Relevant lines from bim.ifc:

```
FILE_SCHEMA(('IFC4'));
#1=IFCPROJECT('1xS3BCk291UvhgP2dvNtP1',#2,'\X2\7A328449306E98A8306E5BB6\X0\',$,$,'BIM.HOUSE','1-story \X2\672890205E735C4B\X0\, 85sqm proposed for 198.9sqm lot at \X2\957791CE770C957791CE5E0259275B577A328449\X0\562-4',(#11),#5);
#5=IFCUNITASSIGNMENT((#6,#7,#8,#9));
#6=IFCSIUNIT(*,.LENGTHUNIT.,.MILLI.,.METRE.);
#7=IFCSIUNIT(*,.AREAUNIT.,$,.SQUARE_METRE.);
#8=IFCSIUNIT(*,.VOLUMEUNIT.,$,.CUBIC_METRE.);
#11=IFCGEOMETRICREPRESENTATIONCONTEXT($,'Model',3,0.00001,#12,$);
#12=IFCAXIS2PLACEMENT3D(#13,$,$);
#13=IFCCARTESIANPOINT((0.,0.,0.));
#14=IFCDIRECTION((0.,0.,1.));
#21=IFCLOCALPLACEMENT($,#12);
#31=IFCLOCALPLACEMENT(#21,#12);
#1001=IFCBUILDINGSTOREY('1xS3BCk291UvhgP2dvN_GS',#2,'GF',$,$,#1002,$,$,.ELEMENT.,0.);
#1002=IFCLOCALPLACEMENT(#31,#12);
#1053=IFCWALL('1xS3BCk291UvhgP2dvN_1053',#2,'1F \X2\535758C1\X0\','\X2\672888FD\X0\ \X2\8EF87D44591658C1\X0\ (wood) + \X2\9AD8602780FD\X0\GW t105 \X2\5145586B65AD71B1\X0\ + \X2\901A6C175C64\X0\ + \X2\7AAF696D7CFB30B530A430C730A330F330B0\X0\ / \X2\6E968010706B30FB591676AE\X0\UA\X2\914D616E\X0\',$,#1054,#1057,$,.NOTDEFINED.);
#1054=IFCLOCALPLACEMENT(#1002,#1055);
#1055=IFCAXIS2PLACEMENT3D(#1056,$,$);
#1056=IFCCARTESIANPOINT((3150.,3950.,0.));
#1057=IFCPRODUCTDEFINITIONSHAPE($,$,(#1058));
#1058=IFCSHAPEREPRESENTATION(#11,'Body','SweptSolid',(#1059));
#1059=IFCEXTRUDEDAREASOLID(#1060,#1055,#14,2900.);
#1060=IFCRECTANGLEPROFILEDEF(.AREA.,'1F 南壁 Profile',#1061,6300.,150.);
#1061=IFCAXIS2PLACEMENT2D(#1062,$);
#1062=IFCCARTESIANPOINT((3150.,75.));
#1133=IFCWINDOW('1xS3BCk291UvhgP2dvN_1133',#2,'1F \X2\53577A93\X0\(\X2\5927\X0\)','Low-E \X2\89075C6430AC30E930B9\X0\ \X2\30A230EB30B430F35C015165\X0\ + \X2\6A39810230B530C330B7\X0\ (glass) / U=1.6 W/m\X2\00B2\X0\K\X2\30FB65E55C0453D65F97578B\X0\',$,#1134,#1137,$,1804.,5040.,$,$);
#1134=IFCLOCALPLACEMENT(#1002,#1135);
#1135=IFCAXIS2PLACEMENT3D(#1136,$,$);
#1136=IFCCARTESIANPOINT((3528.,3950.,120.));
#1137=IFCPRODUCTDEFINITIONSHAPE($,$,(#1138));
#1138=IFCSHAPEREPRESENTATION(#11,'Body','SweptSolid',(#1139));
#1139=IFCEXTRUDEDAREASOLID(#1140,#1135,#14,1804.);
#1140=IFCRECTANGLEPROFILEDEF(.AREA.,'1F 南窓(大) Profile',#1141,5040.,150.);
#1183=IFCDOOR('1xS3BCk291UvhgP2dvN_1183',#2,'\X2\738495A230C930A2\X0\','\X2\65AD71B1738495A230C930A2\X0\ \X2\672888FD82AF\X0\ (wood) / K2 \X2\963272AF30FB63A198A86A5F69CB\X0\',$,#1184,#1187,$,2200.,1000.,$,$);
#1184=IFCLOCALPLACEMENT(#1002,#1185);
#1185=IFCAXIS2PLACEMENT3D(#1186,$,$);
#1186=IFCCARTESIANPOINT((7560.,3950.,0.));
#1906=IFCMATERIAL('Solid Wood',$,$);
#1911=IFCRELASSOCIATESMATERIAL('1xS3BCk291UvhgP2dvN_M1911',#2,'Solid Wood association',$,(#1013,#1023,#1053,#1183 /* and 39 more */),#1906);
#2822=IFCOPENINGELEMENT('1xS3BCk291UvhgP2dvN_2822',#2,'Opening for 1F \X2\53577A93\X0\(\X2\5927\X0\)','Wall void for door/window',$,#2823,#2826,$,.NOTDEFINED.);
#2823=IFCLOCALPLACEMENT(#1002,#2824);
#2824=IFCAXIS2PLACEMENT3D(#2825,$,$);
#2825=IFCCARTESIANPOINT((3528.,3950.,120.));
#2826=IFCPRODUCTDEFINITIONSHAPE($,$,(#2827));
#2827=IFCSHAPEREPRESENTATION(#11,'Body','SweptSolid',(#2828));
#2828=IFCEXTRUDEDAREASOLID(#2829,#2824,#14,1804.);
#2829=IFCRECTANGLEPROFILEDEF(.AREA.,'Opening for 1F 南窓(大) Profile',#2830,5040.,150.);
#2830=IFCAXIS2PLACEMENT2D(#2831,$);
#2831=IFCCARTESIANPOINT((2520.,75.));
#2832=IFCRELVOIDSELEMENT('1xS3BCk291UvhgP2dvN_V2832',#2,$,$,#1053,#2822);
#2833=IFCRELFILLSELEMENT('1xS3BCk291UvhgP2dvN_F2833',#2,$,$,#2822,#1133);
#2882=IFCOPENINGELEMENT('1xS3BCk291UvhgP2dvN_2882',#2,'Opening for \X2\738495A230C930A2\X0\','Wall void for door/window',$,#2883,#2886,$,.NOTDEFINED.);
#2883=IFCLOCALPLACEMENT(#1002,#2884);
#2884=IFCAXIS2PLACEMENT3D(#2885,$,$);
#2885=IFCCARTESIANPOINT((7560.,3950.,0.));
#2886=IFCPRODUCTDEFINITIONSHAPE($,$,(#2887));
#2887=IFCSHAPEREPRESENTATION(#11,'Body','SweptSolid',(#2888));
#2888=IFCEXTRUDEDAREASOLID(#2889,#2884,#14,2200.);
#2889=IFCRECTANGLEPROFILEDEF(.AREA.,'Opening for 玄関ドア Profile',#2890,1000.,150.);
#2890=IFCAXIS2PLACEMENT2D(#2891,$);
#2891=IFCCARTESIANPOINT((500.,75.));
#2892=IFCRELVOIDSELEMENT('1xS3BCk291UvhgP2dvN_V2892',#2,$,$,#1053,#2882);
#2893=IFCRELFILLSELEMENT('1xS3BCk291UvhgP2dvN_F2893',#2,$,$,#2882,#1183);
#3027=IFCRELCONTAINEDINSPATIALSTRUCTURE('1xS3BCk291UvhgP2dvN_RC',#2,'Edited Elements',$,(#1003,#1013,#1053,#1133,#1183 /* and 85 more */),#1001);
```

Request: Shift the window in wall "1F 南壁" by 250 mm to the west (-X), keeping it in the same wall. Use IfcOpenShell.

```python
import ifcopenshell
import ifcopenshell.api.geometry
import ifcopenshell.util.placement

model = ifcopenshell.open("bim.ifc")

window = model.by_guid("1xS3BCk291UvhgP2dvN_1133")
opening = window.FillsVoids[0].RelatingOpeningElement
wall = opening.VoidsElements[0].RelatingBuildingElement

wall_matrix = ifcopenshell.util.placement.get_local_placement(wall.ObjectPlacement)
shift = wall_matrix[:3, 0] * -250.0
before = ifcopenshell.util.placement.get_local_placement(window.ObjectPlacement)[:3, 3].copy()

# The window is not placed relative to its opening, so move both.
for product in (opening, window):
    matrix = ifcopenshell.util.placement.get_local_placement(product.ObjectPlacement)
    matrix[:3, 3] += shift
    ifcopenshell.api.geometry.edit_object_placement(model, product=product, matrix=matrix, is_si=False)

after = ifcopenshell.util.placement.get_local_placement(window.ObjectPlacement)[:3, 3]
print("window moved by", (after - before).round(3) + 0.0)

model.write("bim_rev.ifc")
```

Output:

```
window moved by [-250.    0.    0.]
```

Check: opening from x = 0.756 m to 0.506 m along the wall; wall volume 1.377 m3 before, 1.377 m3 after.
